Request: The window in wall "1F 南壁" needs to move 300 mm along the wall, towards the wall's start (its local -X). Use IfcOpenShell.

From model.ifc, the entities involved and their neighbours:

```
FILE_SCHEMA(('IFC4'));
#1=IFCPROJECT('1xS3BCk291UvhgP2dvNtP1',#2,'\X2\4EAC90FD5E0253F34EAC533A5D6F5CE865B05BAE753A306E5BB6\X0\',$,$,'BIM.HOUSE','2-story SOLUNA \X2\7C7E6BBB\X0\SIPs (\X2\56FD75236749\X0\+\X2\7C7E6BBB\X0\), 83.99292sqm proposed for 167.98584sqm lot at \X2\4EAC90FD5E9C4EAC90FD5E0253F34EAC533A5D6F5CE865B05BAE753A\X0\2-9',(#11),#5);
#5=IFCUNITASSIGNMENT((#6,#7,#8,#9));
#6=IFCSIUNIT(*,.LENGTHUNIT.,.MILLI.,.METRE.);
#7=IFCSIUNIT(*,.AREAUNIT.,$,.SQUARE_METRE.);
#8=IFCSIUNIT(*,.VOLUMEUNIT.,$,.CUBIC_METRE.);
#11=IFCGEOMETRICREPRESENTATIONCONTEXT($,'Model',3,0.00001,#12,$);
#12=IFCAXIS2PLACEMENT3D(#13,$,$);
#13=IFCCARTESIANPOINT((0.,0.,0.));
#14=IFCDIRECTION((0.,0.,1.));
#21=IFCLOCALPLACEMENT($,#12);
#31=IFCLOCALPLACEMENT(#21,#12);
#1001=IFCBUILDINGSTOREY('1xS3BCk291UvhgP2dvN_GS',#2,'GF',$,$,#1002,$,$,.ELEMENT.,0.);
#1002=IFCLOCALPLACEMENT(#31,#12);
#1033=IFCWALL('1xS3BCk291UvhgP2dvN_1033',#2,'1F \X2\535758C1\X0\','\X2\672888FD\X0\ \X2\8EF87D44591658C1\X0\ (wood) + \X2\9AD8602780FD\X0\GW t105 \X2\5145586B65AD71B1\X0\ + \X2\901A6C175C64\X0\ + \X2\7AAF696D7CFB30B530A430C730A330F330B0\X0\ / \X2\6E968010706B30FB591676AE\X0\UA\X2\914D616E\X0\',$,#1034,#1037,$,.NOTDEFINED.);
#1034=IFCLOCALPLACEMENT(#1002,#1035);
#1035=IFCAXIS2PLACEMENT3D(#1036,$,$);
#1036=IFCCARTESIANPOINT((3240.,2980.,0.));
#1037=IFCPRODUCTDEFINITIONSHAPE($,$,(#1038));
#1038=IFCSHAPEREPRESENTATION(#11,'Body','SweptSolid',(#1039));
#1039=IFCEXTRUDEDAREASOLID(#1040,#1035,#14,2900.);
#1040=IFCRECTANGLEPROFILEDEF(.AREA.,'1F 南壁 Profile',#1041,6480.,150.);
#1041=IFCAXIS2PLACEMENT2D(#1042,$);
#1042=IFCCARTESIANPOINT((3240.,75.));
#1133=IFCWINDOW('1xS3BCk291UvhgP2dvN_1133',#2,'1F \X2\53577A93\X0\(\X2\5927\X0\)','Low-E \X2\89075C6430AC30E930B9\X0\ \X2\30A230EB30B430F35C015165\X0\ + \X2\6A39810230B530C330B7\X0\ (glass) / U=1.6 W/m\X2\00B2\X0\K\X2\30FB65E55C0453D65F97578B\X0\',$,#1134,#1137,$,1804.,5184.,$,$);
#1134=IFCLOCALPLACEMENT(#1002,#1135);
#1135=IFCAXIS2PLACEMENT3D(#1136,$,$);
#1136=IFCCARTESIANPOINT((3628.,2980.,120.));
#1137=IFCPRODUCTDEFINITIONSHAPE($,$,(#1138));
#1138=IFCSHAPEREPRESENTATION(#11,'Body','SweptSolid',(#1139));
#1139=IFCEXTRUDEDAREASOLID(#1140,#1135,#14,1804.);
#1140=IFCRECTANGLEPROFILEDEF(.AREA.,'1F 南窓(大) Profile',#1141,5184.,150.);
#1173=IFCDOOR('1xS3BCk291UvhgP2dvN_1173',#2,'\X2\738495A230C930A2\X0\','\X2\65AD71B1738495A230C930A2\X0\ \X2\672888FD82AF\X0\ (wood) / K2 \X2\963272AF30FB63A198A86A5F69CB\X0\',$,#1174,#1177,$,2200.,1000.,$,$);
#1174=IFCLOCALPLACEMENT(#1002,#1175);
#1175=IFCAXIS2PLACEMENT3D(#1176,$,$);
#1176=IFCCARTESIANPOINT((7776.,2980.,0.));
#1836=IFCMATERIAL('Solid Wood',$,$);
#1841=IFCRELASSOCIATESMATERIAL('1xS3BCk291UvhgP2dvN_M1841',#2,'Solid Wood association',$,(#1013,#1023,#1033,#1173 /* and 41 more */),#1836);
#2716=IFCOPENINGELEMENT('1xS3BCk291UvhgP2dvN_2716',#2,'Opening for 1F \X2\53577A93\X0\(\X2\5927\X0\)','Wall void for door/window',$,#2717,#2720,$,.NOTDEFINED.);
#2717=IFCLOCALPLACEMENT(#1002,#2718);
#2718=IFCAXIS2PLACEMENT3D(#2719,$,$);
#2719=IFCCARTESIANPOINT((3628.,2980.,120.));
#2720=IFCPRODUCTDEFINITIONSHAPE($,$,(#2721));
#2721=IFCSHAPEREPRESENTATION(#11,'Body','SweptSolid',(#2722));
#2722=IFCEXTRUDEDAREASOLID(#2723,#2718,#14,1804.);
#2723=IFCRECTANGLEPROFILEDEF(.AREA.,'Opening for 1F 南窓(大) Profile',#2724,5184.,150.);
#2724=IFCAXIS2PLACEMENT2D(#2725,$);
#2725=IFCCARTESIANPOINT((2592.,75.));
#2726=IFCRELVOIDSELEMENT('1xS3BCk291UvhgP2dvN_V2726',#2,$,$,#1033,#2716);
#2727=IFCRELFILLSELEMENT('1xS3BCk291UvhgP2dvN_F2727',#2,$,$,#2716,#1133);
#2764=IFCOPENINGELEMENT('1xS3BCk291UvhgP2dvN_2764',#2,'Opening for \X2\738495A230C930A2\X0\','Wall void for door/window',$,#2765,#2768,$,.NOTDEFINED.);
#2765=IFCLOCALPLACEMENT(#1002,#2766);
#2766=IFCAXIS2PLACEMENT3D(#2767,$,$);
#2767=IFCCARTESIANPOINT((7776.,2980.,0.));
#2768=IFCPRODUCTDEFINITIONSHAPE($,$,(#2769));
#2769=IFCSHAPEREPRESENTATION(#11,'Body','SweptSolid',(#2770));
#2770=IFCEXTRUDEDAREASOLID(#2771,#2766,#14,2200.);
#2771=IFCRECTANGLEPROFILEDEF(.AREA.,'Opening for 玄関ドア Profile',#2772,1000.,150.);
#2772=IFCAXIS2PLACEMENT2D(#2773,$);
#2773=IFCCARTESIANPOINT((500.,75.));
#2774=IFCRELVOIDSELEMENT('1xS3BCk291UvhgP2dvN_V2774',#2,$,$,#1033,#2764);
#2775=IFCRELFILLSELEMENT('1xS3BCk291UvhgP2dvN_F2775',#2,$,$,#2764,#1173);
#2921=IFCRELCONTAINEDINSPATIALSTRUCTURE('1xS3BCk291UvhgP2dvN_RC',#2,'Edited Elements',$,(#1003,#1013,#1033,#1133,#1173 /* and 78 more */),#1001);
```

```python
import ifcopenshell
import ifcopenshell.api.geometry
import ifcopenshell.util.placement
import ifcopenshell.util.unit

model = ifcopenshell.open("model.ifc")
unit_scale = ifcopenshell.util.unit.calculate_unit_scale(model)

window = model.by_guid("1xS3BCk291UvhgP2dvN_1133")
opening = window.FillsVoids[0].RelatingOpeningElement
wall = opening.VoidsElements[0].RelatingBuildingElement

wall_matrix = ifcopenshell.util.placement.get_local_placement(wall.ObjectPlacement)
shift = wall_matrix[:3, 0] * -0.3 / unit_scale
before = ifcopenshell.util.placement.get_local_placement(window.ObjectPlacement)[:3, 3].copy()

# The window is not placed relative to its opening, so move both.
for product in (opening, window):
    matrix = ifcopenshell.util.placement.get_local_placement(product.ObjectPlacement)
    matrix[:3, 3] += shift
    ifcopenshell.api.geometry.edit_object_placement(model, product=product, matrix=matrix, is_si=False)

after = ifcopenshell.util.placement.get_local_placement(window.ObjectPlacement)[:3, 3]
print("window moved by", (after - before).round(3) + 0.0)

model.write("model_v2.ifc")
```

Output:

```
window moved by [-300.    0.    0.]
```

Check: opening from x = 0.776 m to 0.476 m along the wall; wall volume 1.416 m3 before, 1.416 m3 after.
